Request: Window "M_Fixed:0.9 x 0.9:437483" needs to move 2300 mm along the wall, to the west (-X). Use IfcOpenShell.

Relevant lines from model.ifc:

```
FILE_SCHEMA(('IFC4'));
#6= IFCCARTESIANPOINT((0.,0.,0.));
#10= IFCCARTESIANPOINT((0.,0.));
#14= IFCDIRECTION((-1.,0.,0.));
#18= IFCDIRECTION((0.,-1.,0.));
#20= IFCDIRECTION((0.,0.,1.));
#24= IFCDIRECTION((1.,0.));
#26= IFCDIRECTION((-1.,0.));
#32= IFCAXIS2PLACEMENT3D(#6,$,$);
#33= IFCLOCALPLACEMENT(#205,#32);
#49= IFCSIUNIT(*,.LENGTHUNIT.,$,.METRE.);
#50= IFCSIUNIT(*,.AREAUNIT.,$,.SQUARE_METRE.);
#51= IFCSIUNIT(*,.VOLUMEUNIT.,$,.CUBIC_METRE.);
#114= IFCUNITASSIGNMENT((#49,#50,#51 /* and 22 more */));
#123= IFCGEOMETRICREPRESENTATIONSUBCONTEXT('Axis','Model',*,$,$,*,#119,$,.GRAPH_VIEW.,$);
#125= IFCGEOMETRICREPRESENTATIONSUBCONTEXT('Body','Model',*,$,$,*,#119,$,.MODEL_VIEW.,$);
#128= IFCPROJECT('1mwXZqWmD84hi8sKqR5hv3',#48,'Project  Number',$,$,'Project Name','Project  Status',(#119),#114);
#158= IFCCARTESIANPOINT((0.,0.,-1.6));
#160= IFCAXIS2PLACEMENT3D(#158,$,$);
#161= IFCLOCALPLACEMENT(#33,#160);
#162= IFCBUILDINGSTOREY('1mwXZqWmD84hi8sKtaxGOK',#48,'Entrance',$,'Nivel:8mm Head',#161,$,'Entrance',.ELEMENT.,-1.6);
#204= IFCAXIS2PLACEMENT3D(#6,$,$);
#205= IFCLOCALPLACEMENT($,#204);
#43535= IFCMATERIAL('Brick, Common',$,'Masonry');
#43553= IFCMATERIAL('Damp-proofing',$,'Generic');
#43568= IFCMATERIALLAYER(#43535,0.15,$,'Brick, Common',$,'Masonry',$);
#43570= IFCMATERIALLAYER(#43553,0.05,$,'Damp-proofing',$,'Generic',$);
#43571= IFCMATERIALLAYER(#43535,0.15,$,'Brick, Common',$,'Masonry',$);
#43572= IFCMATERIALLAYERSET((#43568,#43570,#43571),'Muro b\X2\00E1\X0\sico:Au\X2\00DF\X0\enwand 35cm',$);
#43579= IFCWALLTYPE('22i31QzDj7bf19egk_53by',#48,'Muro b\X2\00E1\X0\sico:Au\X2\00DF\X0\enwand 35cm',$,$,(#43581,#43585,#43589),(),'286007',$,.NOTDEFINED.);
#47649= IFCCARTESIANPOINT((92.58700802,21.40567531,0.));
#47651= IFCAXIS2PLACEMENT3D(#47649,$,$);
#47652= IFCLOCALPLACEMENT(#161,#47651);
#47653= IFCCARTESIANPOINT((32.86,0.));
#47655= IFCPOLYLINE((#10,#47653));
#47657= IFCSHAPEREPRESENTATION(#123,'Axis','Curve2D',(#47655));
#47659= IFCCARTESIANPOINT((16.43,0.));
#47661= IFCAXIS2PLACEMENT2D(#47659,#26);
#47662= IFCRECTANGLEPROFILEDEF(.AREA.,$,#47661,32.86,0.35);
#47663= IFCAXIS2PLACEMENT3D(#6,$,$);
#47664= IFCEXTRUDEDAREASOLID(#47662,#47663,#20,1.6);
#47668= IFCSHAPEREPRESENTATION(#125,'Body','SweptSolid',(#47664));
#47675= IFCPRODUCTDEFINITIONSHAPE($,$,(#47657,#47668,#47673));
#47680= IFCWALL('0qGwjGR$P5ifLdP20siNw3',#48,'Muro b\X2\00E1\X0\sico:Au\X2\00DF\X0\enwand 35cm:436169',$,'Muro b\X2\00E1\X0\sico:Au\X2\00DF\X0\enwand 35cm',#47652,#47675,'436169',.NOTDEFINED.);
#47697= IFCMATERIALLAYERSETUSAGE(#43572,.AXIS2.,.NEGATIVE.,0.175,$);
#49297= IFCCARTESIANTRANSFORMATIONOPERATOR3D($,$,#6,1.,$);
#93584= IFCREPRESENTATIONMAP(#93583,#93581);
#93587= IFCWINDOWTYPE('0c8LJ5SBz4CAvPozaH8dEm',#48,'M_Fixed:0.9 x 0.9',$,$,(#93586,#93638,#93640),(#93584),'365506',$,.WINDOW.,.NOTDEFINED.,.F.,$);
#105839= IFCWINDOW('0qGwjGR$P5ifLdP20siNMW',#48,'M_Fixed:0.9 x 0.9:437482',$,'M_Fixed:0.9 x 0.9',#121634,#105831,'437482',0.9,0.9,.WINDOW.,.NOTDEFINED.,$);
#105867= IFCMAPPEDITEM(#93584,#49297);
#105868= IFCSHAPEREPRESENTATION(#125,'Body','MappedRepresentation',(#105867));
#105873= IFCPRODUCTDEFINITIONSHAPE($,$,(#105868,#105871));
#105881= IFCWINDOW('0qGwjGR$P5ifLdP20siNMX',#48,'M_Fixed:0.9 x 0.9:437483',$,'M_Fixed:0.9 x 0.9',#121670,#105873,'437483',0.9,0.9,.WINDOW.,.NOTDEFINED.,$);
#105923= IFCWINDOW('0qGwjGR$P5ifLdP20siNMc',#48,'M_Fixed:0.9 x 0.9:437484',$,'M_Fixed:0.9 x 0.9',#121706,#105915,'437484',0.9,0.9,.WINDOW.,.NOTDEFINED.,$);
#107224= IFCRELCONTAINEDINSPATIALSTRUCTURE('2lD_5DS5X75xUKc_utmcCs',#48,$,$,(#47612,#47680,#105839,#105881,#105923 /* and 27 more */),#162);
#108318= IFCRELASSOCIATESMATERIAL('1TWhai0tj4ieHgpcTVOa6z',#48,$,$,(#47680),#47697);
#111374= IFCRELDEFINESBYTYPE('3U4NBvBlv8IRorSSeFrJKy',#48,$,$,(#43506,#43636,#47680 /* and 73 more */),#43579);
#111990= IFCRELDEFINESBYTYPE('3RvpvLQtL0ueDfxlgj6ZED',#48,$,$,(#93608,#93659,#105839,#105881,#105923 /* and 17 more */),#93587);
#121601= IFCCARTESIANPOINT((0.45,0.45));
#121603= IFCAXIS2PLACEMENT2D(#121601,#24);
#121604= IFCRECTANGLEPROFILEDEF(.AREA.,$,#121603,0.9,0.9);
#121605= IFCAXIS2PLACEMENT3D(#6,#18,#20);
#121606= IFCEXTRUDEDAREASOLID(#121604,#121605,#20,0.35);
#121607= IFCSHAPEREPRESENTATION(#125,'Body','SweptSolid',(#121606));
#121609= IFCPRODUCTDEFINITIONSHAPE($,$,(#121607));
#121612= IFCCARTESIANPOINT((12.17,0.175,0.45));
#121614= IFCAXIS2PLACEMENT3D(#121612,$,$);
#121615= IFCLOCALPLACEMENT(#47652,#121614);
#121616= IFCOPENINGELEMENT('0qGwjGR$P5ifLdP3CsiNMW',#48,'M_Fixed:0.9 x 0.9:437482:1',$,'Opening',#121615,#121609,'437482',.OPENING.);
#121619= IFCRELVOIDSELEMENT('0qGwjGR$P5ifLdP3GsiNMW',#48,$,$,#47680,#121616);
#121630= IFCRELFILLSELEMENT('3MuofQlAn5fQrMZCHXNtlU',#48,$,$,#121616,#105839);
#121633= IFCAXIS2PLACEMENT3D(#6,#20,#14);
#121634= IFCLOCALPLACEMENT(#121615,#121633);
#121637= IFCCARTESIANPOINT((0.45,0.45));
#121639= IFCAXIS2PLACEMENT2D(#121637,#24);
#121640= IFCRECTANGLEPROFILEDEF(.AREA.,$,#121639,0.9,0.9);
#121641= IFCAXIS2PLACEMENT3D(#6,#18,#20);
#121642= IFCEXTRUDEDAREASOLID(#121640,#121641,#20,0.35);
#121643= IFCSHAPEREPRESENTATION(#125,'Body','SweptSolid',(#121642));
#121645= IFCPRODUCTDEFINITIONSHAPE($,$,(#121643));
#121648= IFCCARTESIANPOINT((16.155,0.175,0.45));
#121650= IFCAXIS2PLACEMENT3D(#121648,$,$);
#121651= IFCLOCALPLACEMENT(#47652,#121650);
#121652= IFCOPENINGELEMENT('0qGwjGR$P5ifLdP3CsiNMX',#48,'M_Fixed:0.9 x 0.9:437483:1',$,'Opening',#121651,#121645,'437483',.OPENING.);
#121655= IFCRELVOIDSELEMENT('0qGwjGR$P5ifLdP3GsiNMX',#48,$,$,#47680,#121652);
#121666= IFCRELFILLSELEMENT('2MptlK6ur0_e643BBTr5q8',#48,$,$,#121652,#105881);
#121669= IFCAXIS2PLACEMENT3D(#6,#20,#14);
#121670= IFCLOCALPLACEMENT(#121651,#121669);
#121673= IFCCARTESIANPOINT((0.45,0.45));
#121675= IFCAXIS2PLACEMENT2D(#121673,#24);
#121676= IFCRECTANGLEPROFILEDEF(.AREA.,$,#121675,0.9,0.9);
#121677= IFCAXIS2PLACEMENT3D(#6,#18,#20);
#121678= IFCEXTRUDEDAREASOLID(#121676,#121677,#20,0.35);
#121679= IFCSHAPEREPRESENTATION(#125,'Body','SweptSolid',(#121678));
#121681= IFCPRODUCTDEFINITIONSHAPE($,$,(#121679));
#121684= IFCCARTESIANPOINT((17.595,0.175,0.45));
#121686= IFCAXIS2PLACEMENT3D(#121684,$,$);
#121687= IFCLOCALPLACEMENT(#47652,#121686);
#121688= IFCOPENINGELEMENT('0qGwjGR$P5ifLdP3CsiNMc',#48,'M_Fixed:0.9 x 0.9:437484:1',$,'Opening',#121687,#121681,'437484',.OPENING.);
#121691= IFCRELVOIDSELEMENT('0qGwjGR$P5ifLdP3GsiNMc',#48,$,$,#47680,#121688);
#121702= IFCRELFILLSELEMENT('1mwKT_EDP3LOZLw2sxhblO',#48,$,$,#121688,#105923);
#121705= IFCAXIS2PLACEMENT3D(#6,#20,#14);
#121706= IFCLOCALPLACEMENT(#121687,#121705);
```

```python
import ifcopenshell
import ifcopenshell.api.geometry
import ifcopenshell.util.placement

model = ifcopenshell.open("model.ifc")

window = model.by_guid("0qGwjGR$P5ifLdP20siNMX")
opening = window.FillsVoids[0].RelatingOpeningElement
wall = opening.VoidsElements[0].RelatingBuildingElement

wall_matrix = ifcopenshell.util.placement.get_local_placement(wall.ObjectPlacement)
shift = wall_matrix[:3, 0] * -2.3
before = ifcopenshell.util.placement.get_local_placement(window.ObjectPlacement)[:3, 3].copy()

# The window is placed relative to its opening, so it follows when the opening moves.
matrix = ifcopenshell.util.placement.get_local_placement(opening.ObjectPlacement)
matrix[:3, 3] += shift
ifcopenshell.api.geometry.edit_object_placement(
    model, product=opening, matrix=matrix, is_si=False, should_transform_children=True
)

after = ifcopenshell.util.placement.get_local_placement(window.ObjectPlacement)[:3, 3]
print("window moved by", (after - before).round(3) + 0.0)

model.write("model_updated.ifc")
```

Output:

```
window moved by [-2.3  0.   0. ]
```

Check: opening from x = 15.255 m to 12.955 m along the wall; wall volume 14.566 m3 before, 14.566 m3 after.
